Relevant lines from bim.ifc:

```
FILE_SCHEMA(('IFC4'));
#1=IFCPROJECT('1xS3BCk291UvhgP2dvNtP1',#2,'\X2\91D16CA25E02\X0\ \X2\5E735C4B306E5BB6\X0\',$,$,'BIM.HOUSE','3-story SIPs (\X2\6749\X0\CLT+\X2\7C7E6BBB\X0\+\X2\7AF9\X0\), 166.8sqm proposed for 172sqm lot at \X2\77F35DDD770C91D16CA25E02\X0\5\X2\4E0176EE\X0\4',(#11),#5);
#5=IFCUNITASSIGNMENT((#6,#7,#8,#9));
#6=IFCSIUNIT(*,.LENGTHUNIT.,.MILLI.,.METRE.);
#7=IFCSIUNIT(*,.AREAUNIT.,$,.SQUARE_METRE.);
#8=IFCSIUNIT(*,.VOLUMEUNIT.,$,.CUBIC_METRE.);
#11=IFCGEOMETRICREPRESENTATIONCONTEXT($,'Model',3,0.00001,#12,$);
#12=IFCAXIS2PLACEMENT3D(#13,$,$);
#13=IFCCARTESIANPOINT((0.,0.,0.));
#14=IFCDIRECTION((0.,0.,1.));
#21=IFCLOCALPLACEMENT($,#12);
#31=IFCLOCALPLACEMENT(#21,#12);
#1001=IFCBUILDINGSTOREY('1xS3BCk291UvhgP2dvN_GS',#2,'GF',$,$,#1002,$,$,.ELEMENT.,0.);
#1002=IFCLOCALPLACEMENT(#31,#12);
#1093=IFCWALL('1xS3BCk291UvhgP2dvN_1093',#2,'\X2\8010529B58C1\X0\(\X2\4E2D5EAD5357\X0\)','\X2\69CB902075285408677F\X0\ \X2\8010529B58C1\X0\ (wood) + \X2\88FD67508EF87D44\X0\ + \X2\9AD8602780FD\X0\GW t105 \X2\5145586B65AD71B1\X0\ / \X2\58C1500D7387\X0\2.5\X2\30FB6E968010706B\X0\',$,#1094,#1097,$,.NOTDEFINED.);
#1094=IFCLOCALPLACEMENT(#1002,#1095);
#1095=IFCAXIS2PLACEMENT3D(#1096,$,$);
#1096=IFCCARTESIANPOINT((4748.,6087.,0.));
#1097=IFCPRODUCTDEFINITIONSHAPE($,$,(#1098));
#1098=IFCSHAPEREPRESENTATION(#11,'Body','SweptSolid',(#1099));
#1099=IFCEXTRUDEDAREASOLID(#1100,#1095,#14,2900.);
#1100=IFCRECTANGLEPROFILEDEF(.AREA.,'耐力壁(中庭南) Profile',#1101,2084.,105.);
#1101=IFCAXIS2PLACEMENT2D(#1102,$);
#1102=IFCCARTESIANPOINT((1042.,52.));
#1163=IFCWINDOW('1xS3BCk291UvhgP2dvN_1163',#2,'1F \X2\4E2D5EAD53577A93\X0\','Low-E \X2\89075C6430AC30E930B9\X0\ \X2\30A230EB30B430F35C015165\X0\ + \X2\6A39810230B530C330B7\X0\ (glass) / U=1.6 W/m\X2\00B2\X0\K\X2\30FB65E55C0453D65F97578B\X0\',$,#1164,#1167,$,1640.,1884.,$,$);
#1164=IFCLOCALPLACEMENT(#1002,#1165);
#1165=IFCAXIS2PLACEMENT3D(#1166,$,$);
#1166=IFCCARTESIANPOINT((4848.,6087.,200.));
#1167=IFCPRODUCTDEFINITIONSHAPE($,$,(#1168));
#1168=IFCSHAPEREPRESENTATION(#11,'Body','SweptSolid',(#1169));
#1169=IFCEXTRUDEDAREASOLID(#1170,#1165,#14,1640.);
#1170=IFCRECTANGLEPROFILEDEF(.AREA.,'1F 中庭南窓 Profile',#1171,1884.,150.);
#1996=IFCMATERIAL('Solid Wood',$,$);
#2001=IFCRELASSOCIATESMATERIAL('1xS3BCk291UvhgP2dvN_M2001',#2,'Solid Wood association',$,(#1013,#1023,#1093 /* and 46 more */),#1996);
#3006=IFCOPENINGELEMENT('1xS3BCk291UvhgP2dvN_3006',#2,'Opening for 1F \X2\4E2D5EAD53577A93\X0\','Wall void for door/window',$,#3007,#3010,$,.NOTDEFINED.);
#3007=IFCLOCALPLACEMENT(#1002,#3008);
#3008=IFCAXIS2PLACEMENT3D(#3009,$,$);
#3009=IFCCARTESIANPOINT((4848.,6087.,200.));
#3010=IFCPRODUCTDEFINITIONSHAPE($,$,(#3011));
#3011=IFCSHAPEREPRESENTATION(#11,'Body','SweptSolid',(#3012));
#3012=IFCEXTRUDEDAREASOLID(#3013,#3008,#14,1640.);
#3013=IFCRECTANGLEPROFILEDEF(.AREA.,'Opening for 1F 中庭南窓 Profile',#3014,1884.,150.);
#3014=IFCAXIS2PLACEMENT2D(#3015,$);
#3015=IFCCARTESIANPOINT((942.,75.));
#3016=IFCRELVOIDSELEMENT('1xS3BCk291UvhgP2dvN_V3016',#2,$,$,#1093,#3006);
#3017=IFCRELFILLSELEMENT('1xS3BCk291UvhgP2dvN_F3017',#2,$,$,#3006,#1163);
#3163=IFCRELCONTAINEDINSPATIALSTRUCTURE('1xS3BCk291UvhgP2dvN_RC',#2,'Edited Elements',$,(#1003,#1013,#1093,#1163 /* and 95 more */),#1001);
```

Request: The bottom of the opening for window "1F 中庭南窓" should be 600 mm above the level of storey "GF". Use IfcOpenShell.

```python
import numpy as np
import ifcopenshell
import ifcopenshell.api.geometry
import ifcopenshell.geom
import ifcopenshell.util.element
import ifcopenshell.util.placement
import ifcopenshell.util.shape
import ifcopenshell.util.unit

model = ifcopenshell.open("bim.ifc")
unit_scale = ifcopenshell.util.unit.calculate_unit_scale(model)

window = model.by_guid("1xS3BCk291UvhgP2dvN_1163")
opening = window.FillsVoids[0].RelatingOpeningElement
storey = ifcopenshell.util.element.get_container(window, ifc_class="IfcBuildingStorey")
level = ifcopenshell.util.placement.get_local_placement(storey.ObjectPlacement)[2, 3]

# The opening's origin need not be at the sill, so measure its lowest point.
shape = ifcopenshell.geom.create_shape(ifcopenshell.geom.settings(), opening)
bottom = ifcopenshell.util.shape.get_shape_bottom_elevation(shape, shape.geometry) / unit_scale
dz = level + 0.6 / unit_scale - bottom

shift = np.array([0.0, 0.0, dz])
# The window is not placed relative to its opening, so move both.
for product in (opening, window):
    matrix = ifcopenshell.util.placement.get_local_placement(product.ObjectPlacement)
    matrix[:3, 3] += shift
    ifcopenshell.api.geometry.edit_object_placement(model, product=product, matrix=matrix, is_si=False)

print(f"moved by {dz * unit_scale:+.3f} m")

model.write("bim_rev.ifc")
```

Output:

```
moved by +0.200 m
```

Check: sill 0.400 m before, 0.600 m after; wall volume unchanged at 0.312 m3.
